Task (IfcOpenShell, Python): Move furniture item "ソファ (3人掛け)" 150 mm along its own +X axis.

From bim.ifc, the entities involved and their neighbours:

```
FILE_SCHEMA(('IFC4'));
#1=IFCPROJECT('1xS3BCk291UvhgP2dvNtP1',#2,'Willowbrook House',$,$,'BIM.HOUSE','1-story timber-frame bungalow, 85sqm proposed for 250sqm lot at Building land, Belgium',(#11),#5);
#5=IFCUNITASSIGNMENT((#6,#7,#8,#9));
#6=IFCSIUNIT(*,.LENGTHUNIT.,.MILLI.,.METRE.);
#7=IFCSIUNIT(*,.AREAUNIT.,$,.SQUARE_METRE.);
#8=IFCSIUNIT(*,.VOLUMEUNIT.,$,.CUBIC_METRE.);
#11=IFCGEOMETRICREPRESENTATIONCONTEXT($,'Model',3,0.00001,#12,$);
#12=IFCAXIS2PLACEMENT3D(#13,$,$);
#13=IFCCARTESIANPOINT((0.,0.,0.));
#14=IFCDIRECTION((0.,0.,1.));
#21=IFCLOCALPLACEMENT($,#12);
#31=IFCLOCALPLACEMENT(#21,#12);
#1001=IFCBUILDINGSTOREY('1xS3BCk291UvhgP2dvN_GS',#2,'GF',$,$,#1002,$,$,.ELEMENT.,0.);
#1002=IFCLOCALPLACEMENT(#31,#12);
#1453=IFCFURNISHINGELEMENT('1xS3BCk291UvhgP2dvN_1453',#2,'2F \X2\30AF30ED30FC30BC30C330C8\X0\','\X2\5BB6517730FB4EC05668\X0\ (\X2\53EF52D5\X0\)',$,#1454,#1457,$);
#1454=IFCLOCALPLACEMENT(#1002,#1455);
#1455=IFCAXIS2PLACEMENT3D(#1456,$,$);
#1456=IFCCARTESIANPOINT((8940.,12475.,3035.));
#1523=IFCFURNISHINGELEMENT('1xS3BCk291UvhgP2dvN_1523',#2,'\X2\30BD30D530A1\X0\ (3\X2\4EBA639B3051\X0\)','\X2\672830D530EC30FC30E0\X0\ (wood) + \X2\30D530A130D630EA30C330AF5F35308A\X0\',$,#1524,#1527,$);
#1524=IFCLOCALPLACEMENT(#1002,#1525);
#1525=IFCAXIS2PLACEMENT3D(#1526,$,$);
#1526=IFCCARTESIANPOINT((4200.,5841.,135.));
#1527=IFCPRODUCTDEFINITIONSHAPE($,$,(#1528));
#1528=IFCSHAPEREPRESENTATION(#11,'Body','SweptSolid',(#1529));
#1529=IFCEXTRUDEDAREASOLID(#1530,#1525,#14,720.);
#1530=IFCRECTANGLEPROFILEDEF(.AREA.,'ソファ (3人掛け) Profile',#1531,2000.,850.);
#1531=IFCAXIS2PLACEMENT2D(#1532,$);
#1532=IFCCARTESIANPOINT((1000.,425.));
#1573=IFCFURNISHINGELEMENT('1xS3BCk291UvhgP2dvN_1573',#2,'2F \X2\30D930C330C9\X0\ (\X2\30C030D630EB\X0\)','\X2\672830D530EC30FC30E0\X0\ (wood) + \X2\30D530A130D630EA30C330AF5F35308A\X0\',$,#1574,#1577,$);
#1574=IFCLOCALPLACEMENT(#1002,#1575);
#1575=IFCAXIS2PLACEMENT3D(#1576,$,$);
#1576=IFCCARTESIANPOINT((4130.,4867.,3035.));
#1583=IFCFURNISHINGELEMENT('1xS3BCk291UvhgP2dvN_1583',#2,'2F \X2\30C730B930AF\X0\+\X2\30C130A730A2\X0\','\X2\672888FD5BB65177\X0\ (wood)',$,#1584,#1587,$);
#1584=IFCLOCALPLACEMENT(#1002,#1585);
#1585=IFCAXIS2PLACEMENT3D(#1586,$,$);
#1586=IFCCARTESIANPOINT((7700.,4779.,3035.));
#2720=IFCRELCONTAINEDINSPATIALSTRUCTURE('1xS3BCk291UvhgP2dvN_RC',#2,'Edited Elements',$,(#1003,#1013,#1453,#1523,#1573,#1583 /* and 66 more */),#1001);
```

```python
import ifcopenshell
import ifcopenshell.api.geometry
import ifcopenshell.util.placement

model = ifcopenshell.open("bim.ifc")

item = model.by_id(1523)
matrix = ifcopenshell.util.placement.get_local_placement(item.ObjectPlacement)
matrix[:3, 3] += matrix[:3, 0] * 150.0
ifcopenshell.api.geometry.edit_object_placement(model, product=item, matrix=matrix, is_si=False)

print(ifcopenshell.util.placement.get_local_placement(item.ObjectPlacement).round(3) + 0.0)

model.write("bim_v2.ifc")
```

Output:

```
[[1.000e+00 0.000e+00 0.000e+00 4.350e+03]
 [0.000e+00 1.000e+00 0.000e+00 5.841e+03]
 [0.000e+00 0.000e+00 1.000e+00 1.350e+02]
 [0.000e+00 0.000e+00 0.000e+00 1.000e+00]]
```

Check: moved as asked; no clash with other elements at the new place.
